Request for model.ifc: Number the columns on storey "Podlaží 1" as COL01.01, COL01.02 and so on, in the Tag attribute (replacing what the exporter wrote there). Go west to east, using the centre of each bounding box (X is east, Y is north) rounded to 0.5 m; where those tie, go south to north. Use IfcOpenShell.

First a look at what the model holds.

```python
import ifcopenshell
import ifcopenshell.util.element
import ifcopenshell.util.placement

model = ifcopenshell.open("model.ifc")
print(model.schema)
storey = next(s for s in model.by_type("IfcBuildingStorey") if s.Name == "Podlaží 1")
columns = [e for e in ifcopenshell.util.element.get_decomposition(storey) if e.is_a("IfcColumn")]
for e in sorted(columns, key=lambda e: e.id()):
    origin = ifcopenshell.util.placement.get_local_placement(e.ObjectPlacement)[:3, 3]
    print(e.id(), e.Tag, e.Name, origin.round(2) + 0.0, sep=" | ")
```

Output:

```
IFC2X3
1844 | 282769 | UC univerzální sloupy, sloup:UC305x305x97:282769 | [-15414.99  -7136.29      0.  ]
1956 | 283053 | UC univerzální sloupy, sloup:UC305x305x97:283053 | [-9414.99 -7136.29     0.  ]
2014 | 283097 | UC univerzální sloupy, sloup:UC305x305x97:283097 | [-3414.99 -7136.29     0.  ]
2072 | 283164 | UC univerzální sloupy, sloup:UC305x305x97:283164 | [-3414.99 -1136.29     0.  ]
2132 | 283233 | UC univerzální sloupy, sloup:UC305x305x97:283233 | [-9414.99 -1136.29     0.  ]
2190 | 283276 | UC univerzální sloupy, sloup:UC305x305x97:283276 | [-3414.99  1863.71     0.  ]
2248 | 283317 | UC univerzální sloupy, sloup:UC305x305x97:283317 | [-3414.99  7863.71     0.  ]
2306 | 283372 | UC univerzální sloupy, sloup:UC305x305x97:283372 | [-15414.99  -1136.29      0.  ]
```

```python
import ifcopenshell
import ifcopenshell.geom
import ifcopenshell.util.element
import ifcopenshell.util.shape

model = ifcopenshell.open("model.ifc")
settings = ifcopenshell.geom.settings()
settings.set("use-world-coords", True)


def centre(element):
    shape = ifcopenshell.geom.create_shape(settings, element)
    return ifcopenshell.util.shape.get_bbox_centroid(shape.geometry)


storey = next(s for s in model.by_type("IfcBuildingStorey") if s.Name == "Podlaží 1")
columns = [e for e in ifcopenshell.util.element.get_decomposition(storey) if e.is_a("IfcColumn")]

# Insertion points can sit at a corner or the storey origin, so sort by the geometry (in metres).
centres = {e: centre(e) for e in columns}
columns.sort(key=lambda e: (round(centres[e][0] / 0.5), centres[e][1]))

for i, e in enumerate(columns, start=1):
    number = f"COL01.{i:02d}"
    e.Tag = number
    print(e.id(), number)

model.write("model_rev.ifc")
```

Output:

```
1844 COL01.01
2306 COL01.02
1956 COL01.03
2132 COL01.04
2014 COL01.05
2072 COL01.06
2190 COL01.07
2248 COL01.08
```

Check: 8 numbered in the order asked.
